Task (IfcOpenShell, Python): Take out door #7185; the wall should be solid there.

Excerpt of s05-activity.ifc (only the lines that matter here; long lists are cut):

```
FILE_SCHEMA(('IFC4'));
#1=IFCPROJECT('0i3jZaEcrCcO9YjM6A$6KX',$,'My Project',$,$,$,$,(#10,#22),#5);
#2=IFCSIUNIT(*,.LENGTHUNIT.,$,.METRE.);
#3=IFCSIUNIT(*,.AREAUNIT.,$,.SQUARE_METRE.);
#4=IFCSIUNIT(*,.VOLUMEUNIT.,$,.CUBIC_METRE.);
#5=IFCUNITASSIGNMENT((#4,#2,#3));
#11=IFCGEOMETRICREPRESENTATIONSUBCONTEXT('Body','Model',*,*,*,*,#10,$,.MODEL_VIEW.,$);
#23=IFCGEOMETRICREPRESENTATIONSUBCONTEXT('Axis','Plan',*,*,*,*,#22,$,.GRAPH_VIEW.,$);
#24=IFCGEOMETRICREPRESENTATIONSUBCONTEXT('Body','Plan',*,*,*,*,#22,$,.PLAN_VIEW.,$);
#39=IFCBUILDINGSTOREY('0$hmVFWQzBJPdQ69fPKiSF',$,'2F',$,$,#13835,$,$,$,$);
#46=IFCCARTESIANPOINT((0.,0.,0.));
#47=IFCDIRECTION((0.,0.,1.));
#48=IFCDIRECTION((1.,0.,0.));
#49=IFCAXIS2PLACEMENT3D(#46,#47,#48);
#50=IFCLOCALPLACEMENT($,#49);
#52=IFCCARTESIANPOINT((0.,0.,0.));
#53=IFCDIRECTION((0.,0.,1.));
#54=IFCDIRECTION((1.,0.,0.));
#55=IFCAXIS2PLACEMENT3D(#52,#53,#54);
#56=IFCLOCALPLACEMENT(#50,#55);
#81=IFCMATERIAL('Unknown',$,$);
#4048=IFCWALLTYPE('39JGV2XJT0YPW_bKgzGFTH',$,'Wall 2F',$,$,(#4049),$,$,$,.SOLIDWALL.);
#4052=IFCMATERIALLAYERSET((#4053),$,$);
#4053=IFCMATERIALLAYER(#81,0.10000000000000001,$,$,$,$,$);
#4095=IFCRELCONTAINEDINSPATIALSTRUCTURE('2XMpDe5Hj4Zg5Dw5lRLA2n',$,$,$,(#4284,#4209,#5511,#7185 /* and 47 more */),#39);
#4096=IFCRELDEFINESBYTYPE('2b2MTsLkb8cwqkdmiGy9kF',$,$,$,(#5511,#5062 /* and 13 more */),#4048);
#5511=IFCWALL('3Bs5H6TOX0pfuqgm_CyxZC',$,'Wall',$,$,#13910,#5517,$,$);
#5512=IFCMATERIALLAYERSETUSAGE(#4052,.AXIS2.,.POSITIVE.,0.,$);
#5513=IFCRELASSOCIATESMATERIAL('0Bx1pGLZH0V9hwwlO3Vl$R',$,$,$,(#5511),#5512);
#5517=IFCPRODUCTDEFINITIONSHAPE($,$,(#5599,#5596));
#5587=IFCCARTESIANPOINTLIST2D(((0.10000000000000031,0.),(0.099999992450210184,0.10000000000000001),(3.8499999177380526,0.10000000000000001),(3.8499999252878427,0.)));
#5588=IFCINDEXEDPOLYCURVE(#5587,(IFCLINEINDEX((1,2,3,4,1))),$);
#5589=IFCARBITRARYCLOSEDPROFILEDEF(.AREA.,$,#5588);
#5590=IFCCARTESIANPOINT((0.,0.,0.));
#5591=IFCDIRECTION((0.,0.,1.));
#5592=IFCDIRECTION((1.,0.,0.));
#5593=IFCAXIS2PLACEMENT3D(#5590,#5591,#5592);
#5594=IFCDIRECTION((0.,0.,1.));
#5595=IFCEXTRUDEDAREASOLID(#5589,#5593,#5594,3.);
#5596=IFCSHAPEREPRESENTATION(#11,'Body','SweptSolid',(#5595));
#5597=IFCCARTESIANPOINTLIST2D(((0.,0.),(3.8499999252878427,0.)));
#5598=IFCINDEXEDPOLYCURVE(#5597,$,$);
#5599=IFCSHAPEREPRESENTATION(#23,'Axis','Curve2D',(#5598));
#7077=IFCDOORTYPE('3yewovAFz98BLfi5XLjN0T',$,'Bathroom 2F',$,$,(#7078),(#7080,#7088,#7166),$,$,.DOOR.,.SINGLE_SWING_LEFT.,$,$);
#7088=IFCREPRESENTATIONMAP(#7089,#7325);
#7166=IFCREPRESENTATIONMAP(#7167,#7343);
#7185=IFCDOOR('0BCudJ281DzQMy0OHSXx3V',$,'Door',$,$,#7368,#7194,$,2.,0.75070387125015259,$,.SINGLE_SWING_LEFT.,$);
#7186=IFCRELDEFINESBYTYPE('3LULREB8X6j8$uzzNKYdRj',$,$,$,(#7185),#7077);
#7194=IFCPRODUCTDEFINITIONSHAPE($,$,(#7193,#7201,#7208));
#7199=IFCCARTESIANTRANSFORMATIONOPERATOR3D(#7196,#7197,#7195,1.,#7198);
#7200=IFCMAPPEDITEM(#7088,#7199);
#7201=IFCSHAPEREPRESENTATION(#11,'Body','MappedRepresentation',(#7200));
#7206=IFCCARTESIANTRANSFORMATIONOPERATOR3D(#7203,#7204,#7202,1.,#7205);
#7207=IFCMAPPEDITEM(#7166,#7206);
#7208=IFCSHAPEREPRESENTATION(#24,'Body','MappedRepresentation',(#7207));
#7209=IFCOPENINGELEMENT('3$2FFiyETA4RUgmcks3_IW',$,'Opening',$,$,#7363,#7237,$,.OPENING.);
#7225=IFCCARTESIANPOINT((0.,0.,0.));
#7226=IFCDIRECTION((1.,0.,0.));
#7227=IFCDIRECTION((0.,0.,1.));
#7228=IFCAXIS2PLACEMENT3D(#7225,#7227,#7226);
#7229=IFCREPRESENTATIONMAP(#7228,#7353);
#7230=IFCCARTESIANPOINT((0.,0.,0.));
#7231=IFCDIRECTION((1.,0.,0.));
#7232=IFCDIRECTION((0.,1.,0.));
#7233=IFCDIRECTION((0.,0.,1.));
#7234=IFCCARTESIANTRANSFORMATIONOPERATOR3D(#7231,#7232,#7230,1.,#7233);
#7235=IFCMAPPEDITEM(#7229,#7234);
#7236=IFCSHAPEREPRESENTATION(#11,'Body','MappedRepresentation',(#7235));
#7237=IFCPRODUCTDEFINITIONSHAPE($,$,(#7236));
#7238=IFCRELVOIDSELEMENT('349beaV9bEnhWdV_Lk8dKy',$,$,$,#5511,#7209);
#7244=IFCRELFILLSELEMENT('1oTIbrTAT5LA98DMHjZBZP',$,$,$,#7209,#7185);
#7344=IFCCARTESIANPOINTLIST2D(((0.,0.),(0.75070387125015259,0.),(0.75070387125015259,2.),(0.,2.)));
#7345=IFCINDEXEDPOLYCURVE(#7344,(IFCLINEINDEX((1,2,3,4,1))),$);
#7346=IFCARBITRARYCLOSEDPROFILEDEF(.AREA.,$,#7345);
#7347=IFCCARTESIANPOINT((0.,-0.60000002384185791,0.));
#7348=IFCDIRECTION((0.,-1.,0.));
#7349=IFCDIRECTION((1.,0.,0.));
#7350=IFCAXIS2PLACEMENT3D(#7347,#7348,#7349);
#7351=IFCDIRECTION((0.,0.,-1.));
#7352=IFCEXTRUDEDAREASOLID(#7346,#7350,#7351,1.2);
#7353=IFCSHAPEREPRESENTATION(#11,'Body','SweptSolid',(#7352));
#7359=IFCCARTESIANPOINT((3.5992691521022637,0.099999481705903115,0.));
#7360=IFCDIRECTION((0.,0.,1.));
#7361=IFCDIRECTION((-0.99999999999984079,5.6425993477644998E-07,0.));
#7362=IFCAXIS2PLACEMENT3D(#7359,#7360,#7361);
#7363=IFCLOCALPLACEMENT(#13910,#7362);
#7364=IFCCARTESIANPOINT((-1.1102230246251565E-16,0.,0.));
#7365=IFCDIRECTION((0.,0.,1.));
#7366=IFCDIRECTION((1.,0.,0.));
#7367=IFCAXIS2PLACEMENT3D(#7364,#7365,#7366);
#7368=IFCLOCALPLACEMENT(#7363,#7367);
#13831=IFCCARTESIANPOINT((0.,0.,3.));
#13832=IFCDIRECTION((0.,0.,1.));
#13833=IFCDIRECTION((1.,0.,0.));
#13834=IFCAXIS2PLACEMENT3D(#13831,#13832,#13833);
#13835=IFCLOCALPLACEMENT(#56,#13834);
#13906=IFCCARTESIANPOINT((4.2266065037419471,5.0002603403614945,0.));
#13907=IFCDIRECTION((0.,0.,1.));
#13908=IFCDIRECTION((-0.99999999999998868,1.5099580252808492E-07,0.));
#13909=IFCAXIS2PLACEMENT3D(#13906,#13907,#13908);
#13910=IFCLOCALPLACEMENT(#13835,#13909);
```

```python
import ifcopenshell
import ifcopenshell.api.feature
import ifcopenshell.api.root
import ifcopenshell.geom
import ifcopenshell.util.shape

model = ifcopenshell.open("s05-activity.ifc")
settings = ifcopenshell.geom.settings()


def volume(element):
    """Net volume in cubic metres, openings subtracted."""
    shape = ifcopenshell.geom.create_shape(settings, element)
    return ifcopenshell.util.shape.get_volume(shape.geometry)


door = model.by_guid("0BCudJ281DzQMy0OHSXx3V")
opening = door.FillsVoids[0].RelatingOpeningElement
wall = opening.VoidsElements[0].RelatingBuildingElement
before = volume(wall)

ifcopenshell.api.root.remove_product(model, product=door)
ifcopenshell.api.feature.remove_feature(model, feature=opening)

after = volume(wall)

print(f"wall volume {before:.3f} -> {after:.3f} m3")

model.write("s05-activity_edited.ifc")
```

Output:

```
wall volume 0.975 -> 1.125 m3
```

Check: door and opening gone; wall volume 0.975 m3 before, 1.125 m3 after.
